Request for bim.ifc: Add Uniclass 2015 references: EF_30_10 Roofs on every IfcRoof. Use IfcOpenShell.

First a look at what the model holds.

```python
import ifcopenshell

model = ifcopenshell.open("bim.ifc")
print(model.schema)
print("classifications:", [c.Name for c in model.by_type("IfcClassification")])
for ifc_class in ("IfcDoor", "IfcRoof", "IfcStair", "IfcWall", "IfcWindow"):
    print(ifc_class, len(model.by_type(ifc_class)))
```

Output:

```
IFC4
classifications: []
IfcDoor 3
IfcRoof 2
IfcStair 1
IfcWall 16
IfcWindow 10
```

```python
import ifcopenshell
import ifcopenshell.api.classification

model = ifcopenshell.open("bim.ifc")

system = ifcopenshell.api.classification.add_classification(model, classification="Uniclass 2015")

codes = {
    "IfcRoof": ("EF_30_10", "Roofs"),
}
for ifc_class, (code, name) in codes.items():
    products = model.by_type(ifc_class)
    ifcopenshell.api.classification.add_reference(
        model, products=products, classification=system, identification=code, name=name
    )
    print(code, len(products))

model.write("bim-out.ifc")
```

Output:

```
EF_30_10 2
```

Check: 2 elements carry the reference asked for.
